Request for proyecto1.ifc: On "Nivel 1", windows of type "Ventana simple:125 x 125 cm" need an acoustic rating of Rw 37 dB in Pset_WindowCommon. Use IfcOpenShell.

First a look at what the model holds.

```python
import ifcopenshell
import ifcopenshell.util.element

model = ifcopenshell.open("proyecto1.ifc")
print(model.schema)
storey = next(s for s in model.by_type("IfcBuildingStorey") if s.Name == "Nivel 1")
windows = [e for e in ifcopenshell.util.element.get_decomposition(storey) if e.is_a("IfcWindow")]
seen = {}
for e in windows:
    element_type = ifcopenshell.util.element.get_type(e)
    key = (element_type.Name if element_type != e and element_type else None, ifcopenshell.util.element.get_pset(e, "Pset_WindowCommon", "AcousticRating"))
    seen[key] = seen.get(key, 0) + 1
for (name, value), count in sorted(seen.items(), key=str):
    print(count, "x", name, "|", value)
```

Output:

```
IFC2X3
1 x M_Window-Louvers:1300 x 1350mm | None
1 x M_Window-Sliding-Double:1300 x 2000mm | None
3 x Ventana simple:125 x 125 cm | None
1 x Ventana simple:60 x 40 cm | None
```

```python
import ifcopenshell
import ifcopenshell.api.pset
import ifcopenshell.util.element

model = ifcopenshell.open("proyecto1.ifc")

storey = next(s for s in model.by_type("IfcBuildingStorey") if s.Name == "Nivel 1")
windows = [e for e in ifcopenshell.util.element.get_decomposition(storey) if e.is_a("IfcWindow")]

count = 0
for e in windows:
    element_type = ifcopenshell.util.element.get_type(e)
    if element_type in (None, e) or element_type.Name != "Ventana simple:125 x 125 cm":
        continue
    # add_pset returns the element's existing set when there is one.
    pset = ifcopenshell.api.pset.add_pset(model, product=e, name="Pset_WindowCommon")
    ifcopenshell.api.pset.edit_pset(model, pset=pset, properties={"AcousticRating": "Rw 37 dB"})
    count += 1

print(count, "windows updated")

model.write("proyecto1_v2.ifc")
```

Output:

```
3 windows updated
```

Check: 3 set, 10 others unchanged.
